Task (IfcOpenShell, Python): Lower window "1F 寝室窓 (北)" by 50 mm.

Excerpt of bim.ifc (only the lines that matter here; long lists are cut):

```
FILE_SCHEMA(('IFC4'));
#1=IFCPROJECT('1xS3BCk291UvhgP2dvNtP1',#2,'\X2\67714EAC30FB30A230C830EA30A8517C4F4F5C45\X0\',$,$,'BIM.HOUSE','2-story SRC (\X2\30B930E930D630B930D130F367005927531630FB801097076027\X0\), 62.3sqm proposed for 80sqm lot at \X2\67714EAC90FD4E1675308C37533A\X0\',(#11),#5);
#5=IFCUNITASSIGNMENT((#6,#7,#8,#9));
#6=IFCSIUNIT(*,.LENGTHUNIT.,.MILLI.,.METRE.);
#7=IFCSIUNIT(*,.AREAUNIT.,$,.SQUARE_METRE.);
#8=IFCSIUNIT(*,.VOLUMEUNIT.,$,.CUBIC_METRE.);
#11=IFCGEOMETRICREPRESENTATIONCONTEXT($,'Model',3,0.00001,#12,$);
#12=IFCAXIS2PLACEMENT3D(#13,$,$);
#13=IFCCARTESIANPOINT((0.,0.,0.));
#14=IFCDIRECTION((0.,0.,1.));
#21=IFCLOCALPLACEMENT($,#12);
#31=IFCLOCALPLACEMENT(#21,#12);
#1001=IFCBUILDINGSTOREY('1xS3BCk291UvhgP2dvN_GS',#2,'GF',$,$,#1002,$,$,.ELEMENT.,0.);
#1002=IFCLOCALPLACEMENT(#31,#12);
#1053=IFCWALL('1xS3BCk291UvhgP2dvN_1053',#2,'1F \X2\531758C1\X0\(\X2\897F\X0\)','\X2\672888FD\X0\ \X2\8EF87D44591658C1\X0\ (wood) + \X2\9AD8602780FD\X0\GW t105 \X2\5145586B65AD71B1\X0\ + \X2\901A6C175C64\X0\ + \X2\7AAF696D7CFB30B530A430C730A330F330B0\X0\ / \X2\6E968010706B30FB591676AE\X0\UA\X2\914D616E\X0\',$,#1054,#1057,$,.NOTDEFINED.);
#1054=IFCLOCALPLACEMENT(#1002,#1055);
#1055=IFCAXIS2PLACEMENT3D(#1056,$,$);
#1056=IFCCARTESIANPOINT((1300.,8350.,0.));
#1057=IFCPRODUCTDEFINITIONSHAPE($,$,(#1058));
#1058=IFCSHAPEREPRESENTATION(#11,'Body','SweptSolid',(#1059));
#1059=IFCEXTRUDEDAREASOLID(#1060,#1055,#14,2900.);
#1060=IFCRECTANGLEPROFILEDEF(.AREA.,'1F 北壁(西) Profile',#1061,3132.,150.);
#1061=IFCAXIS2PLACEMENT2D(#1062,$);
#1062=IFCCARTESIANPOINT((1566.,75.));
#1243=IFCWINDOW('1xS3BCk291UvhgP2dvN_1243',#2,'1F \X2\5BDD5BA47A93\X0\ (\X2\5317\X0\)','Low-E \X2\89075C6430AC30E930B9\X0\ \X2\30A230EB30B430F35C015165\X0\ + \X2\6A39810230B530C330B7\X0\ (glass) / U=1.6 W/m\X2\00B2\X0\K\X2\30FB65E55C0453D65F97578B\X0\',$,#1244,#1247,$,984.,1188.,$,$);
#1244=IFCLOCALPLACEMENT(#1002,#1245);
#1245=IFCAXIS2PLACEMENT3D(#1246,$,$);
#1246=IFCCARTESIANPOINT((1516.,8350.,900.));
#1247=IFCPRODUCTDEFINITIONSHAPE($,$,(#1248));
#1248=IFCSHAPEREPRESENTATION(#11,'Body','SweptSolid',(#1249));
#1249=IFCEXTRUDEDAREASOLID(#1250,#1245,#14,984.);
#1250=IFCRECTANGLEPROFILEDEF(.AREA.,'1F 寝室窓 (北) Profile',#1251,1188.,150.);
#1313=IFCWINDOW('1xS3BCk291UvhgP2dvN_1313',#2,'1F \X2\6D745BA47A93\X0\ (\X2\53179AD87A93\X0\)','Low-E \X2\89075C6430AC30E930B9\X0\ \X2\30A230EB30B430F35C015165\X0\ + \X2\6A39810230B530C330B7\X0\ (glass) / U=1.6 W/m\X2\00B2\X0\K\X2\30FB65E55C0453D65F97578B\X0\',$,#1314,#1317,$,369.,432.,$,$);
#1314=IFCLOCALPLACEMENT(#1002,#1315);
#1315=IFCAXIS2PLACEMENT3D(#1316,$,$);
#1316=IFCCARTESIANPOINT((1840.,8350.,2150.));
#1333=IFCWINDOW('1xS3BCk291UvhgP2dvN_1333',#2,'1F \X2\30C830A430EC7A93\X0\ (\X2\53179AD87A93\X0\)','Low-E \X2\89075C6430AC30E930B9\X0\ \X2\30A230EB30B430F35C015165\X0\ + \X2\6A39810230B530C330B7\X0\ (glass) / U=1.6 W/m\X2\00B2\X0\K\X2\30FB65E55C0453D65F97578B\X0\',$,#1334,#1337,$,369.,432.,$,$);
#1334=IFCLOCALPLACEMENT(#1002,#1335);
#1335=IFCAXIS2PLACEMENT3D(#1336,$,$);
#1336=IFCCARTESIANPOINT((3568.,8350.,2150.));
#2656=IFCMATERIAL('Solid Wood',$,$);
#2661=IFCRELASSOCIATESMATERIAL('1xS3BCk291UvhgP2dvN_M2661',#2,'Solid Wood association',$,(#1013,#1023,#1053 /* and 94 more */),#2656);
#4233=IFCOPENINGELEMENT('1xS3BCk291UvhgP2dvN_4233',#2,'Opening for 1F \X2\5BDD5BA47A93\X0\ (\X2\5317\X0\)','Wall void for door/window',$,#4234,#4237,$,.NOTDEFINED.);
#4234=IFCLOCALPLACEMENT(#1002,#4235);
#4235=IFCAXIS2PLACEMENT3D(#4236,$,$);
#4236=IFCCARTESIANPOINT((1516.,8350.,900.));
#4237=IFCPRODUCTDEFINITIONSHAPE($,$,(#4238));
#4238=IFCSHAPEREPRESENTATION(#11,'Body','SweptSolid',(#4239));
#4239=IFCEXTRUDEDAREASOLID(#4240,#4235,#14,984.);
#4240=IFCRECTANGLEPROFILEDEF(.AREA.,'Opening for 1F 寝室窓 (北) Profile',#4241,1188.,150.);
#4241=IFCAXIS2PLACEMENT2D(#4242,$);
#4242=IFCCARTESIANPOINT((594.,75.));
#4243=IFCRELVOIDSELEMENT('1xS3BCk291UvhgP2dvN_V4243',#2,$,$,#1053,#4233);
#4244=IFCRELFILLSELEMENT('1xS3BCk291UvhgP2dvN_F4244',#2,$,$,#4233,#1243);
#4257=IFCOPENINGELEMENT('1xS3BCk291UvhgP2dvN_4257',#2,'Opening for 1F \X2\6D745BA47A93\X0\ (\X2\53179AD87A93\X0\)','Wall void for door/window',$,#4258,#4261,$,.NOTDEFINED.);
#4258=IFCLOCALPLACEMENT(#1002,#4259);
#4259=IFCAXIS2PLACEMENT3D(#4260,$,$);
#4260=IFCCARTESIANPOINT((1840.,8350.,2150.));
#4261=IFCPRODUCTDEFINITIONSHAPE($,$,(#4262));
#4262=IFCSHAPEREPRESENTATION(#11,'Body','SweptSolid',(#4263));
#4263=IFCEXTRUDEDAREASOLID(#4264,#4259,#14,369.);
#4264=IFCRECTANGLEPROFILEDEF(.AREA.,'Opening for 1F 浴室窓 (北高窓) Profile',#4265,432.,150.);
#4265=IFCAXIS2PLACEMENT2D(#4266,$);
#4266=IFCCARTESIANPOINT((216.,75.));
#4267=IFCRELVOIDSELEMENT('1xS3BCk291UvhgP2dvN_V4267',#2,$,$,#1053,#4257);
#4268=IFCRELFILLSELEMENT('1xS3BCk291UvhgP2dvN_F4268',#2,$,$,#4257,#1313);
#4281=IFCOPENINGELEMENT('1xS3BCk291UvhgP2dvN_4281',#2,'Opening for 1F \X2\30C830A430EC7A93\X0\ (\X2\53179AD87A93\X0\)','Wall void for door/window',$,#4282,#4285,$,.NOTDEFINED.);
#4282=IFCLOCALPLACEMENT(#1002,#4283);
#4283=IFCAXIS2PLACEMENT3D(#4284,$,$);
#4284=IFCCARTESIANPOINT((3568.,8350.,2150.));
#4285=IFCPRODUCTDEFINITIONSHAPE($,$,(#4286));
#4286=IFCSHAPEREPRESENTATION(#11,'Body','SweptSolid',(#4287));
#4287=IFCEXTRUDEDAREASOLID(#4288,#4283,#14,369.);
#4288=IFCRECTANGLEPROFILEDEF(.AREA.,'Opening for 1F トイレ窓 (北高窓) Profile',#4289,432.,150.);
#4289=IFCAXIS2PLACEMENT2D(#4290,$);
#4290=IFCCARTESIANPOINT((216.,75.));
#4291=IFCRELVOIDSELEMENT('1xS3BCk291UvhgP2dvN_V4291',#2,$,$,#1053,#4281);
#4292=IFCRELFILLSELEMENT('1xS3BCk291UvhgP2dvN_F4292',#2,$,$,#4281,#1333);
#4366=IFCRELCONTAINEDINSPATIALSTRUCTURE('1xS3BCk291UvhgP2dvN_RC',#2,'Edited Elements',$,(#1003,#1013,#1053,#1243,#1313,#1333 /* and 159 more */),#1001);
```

```python
import numpy as np
import ifcopenshell
import ifcopenshell.api.geometry
import ifcopenshell.util.placement
import ifcopenshell.util.unit

model = ifcopenshell.open("bim.ifc")
unit_scale = ifcopenshell.util.unit.calculate_unit_scale(model)

window = model.by_id(1243)
opening = window.FillsVoids[0].RelatingOpeningElement
dz = -50.0

shift = np.array([0.0, 0.0, dz])
# The window is not placed relative to its opening, so move both.
for product in (opening, window):
    matrix = ifcopenshell.util.placement.get_local_placement(product.ObjectPlacement)
    matrix[:3, 3] += shift
    ifcopenshell.api.geometry.edit_object_placement(model, product=product, matrix=matrix, is_si=False)

print(f"moved by {dz * unit_scale:+.3f} m")

model.write("bim_updated.ifc")
```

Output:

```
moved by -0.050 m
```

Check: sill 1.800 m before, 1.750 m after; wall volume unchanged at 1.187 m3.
